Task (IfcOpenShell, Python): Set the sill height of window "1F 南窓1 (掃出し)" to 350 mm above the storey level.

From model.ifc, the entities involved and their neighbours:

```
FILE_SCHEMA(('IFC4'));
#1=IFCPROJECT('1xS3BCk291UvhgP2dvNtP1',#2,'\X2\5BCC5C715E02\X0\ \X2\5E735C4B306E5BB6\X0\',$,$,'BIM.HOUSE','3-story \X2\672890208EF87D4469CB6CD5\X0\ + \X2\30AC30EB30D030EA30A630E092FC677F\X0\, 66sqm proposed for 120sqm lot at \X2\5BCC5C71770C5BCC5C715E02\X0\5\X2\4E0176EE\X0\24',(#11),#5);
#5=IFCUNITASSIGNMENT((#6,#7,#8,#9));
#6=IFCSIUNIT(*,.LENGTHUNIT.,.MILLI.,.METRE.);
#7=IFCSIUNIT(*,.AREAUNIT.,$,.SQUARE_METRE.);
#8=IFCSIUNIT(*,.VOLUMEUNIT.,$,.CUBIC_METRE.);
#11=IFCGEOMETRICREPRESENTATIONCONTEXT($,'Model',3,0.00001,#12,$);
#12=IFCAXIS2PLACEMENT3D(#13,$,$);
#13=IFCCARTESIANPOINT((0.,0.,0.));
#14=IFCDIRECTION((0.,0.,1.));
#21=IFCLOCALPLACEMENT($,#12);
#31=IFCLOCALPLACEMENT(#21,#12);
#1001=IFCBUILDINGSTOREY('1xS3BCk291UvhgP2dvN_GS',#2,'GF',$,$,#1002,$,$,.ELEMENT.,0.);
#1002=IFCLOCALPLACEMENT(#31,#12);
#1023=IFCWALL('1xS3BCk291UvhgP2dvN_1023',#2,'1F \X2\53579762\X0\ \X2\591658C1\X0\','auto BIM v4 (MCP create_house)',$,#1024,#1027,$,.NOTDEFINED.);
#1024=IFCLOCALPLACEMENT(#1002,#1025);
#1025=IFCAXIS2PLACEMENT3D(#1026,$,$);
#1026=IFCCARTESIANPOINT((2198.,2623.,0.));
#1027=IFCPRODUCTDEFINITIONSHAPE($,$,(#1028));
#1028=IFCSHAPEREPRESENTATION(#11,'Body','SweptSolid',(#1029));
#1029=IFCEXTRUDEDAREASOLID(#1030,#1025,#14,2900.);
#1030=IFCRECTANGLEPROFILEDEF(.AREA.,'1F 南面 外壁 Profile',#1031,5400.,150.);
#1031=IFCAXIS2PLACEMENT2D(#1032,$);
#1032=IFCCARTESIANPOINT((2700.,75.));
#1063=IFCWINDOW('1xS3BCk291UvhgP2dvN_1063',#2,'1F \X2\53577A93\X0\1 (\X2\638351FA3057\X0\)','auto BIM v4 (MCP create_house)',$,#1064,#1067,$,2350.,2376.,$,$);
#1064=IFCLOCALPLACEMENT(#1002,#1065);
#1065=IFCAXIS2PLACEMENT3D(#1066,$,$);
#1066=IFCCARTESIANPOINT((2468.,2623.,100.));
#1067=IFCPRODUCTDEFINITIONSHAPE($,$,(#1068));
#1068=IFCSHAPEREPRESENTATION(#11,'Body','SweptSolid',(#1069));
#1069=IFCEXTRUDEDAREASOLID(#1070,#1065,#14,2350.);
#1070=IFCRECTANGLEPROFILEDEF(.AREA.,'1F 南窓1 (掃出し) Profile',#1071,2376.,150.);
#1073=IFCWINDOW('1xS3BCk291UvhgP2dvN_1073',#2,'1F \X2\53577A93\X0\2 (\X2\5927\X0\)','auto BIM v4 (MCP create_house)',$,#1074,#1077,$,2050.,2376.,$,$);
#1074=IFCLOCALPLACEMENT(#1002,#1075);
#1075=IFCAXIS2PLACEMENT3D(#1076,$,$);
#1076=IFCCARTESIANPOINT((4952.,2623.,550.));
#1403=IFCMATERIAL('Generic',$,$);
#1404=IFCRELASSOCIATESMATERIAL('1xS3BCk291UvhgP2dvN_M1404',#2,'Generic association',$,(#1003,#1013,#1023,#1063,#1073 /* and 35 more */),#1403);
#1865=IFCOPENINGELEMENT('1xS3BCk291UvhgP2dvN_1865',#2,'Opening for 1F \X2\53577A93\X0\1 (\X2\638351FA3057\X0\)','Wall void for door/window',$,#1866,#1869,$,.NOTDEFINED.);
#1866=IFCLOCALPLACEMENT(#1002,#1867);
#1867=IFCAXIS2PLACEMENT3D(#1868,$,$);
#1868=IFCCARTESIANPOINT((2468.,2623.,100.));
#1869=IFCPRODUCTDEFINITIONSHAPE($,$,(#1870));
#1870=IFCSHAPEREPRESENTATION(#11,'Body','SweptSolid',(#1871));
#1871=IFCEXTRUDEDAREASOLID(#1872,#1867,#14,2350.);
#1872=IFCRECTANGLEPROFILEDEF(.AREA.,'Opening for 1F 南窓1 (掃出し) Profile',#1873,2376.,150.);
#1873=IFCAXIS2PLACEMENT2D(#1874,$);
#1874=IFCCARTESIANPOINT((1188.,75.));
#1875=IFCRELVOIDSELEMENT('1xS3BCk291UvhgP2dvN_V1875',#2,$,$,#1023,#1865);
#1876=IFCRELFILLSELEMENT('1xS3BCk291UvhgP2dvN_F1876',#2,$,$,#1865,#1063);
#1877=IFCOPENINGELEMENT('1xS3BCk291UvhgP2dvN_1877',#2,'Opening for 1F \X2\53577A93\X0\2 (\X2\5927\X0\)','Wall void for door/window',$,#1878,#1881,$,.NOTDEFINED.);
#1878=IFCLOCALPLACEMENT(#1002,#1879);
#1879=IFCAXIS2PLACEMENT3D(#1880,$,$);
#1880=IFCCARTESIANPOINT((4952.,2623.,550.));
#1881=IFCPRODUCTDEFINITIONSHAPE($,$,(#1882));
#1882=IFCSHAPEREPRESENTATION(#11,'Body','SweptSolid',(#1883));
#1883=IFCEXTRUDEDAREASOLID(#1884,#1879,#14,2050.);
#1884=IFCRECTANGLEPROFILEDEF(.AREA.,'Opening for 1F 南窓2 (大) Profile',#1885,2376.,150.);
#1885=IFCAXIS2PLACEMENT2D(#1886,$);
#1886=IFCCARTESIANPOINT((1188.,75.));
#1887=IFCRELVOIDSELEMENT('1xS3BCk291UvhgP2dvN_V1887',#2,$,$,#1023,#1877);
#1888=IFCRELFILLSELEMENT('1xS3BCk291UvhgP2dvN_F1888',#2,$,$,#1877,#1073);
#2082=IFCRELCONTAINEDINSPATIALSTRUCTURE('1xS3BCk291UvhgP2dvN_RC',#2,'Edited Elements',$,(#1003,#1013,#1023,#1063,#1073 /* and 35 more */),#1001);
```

```python
import numpy as np
import ifcopenshell
import ifcopenshell.api.geometry
import ifcopenshell.geom
import ifcopenshell.util.element
import ifcopenshell.util.placement
import ifcopenshell.util.shape
import ifcopenshell.util.unit

model = ifcopenshell.open("model.ifc")
unit_scale = ifcopenshell.util.unit.calculate_unit_scale(model)

window = model.by_id(1063)
opening = window.FillsVoids[0].RelatingOpeningElement
storey = ifcopenshell.util.element.get_container(window, ifc_class="IfcBuildingStorey")
level = ifcopenshell.util.placement.get_local_placement(storey.ObjectPlacement)[2, 3]

# The opening's origin need not be at the sill, so measure its lowest point.
shape = ifcopenshell.geom.create_shape(ifcopenshell.geom.settings(), opening)
bottom = ifcopenshell.util.shape.get_shape_bottom_elevation(shape, shape.geometry) / unit_scale
dz = level + 0.35 / unit_scale - bottom

shift = np.array([0.0, 0.0, dz])
# The window is not placed relative to its opening, so move both.
for product in (opening, window):
    matrix = ifcopenshell.util.placement.get_local_placement(product.ObjectPlacement)
    matrix[:3, 3] += shift
    ifcopenshell.api.geometry.edit_object_placement(model, product=product, matrix=matrix, is_si=False)

print(f"moved by {dz * unit_scale:+.3f} m")

model.write("model_edited.ifc")
```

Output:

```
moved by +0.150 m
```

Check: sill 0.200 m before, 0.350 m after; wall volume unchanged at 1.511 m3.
